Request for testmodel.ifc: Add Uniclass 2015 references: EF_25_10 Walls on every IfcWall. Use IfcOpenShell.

First a look at what the model holds.

```python
import ifcopenshell

model = ifcopenshell.open("testmodel.ifc")
print(model.schema)
print("classifications:", [c.Name for c in model.by_type("IfcClassification")])
for ifc_class in ("IfcDoor", "IfcRoof", "IfcStair", "IfcWall", "IfcWindow"):
    print(ifc_class, len(model.by_type(ifc_class)))
```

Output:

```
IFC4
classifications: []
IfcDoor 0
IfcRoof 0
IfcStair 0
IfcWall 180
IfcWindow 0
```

```python
import ifcopenshell
import ifcopenshell.api.classification

model = ifcopenshell.open("testmodel.ifc")

system = ifcopenshell.api.classification.add_classification(model, classification="Uniclass 2015")

codes = {
    "IfcWall": ("EF_25_10", "Walls"),
}
for ifc_class, (code, name) in codes.items():
    products = model.by_type(ifc_class)
    ifcopenshell.api.classification.add_reference(
        model, products=products, classification=system, identification=code, name=name
    )
    print(code, len(products))

model.write("testmodel_edited.ifc")
```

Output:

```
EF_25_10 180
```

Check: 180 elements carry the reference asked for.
